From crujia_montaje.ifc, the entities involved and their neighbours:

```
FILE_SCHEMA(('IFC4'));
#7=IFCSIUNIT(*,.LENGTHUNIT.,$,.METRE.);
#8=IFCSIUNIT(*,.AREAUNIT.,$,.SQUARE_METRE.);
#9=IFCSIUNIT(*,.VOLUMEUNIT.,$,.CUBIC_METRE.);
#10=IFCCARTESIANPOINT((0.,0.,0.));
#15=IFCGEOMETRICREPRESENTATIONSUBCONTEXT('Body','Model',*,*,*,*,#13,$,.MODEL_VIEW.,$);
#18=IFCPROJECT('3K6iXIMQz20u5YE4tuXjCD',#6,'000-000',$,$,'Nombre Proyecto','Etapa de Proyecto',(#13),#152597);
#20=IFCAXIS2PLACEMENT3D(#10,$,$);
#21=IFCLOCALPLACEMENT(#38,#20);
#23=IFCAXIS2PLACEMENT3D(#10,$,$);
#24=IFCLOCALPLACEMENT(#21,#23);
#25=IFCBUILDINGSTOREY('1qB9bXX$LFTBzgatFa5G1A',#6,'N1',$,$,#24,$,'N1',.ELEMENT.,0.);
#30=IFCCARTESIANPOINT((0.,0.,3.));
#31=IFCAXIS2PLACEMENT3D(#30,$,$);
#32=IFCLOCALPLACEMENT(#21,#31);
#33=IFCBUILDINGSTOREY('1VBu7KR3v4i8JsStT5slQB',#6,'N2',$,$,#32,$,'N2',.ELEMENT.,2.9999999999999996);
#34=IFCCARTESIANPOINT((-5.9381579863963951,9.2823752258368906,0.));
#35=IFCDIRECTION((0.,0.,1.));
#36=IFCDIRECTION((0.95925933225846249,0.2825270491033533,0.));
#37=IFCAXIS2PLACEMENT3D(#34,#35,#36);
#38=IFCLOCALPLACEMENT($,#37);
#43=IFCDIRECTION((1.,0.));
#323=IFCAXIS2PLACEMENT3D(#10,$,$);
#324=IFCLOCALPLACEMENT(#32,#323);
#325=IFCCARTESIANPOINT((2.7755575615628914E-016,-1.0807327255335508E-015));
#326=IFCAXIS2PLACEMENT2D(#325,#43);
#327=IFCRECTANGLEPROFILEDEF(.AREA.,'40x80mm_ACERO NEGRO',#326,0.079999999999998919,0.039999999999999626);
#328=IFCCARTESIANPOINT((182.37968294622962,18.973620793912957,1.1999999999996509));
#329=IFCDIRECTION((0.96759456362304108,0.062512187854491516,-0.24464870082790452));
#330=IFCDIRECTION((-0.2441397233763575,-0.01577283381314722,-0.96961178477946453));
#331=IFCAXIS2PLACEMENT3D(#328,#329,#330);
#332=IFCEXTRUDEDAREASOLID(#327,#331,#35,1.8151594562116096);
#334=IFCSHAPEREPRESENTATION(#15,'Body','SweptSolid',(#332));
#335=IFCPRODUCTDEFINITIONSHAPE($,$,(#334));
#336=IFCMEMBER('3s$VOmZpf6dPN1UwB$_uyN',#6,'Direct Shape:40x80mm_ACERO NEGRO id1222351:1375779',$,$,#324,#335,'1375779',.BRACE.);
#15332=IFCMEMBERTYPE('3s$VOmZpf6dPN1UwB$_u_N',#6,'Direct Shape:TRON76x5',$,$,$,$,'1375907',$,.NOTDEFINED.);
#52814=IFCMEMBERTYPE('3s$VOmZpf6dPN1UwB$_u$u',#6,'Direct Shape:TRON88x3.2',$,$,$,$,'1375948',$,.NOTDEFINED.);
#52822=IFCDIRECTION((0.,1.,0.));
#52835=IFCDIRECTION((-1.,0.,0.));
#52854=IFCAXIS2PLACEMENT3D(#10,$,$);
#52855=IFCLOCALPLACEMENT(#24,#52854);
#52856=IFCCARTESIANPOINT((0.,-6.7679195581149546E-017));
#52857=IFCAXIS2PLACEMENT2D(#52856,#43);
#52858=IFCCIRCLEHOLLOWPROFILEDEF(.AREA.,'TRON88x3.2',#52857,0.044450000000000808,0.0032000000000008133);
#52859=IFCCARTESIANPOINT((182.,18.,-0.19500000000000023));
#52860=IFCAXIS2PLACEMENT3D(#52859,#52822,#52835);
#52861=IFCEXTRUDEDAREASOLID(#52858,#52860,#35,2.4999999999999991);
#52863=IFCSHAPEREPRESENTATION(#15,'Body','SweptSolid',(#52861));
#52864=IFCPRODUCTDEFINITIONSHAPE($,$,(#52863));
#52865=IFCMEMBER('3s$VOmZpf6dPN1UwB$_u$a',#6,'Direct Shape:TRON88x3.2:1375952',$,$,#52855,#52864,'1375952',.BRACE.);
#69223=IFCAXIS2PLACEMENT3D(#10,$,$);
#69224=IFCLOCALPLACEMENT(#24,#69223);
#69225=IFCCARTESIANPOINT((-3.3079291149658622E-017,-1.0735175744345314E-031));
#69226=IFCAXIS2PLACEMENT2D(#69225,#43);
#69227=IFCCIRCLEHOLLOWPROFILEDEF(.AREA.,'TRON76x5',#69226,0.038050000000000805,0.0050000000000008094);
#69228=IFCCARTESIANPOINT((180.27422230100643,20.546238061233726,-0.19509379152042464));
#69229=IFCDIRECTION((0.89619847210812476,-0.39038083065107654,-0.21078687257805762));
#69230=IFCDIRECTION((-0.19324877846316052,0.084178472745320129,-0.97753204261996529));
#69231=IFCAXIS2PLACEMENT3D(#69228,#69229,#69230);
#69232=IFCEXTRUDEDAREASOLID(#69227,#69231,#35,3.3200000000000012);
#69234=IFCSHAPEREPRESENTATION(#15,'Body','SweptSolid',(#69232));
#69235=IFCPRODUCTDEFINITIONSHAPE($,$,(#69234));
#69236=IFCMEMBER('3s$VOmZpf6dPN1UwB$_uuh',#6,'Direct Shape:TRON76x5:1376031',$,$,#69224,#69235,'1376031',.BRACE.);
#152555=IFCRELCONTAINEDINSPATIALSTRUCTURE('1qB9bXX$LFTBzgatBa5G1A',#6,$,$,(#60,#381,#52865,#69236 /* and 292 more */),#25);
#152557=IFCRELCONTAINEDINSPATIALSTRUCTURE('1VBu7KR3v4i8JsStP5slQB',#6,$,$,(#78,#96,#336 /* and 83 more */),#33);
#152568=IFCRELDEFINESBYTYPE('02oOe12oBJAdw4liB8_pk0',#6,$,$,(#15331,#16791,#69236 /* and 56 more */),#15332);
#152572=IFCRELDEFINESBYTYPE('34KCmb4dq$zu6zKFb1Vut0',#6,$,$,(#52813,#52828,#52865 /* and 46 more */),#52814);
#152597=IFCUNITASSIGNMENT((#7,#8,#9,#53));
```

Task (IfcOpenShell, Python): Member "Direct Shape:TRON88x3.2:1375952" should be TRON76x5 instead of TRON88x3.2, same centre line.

```python
import ifcopenshell
import ifcopenshell.api.type
import ifcopenshell.util.element
import ifcopenshell.util.representation

model = ifcopenshell.open("crujia_montaje.ifc")

member = model.by_id(52865)
source = next(p for p in model.by_type("IfcCircleHollowProfileDef") if p.ProfileName == "TRON76x5")

body = ifcopenshell.util.representation.get_representation(member, "Model", "Body")
solid = body.Items[0]
old_profile = solid.SweptArea

# Copy the section's sizes but keep this member's own profile position.
profile = ifcopenshell.util.element.copy(model, source)
profile.Position = old_profile.Position
solid.SweptArea = profile
if not model.get_total_inverses(old_profile):
    ifcopenshell.util.element.remove_deep2(model, old_profile)

new_type = model.by_id(15332)
ifcopenshell.api.type.assign_type(
    model, related_objects=[member], relating_type=new_type, should_map_representations=False
)
member.Name = member.Name.replace("TRON88x3.2", "TRON76x5")

print(solid.SweptArea)

model.write("crujia_montaje-out.ifc")
```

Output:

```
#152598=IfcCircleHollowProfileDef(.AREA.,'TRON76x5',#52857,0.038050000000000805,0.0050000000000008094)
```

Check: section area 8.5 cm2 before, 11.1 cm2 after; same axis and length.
